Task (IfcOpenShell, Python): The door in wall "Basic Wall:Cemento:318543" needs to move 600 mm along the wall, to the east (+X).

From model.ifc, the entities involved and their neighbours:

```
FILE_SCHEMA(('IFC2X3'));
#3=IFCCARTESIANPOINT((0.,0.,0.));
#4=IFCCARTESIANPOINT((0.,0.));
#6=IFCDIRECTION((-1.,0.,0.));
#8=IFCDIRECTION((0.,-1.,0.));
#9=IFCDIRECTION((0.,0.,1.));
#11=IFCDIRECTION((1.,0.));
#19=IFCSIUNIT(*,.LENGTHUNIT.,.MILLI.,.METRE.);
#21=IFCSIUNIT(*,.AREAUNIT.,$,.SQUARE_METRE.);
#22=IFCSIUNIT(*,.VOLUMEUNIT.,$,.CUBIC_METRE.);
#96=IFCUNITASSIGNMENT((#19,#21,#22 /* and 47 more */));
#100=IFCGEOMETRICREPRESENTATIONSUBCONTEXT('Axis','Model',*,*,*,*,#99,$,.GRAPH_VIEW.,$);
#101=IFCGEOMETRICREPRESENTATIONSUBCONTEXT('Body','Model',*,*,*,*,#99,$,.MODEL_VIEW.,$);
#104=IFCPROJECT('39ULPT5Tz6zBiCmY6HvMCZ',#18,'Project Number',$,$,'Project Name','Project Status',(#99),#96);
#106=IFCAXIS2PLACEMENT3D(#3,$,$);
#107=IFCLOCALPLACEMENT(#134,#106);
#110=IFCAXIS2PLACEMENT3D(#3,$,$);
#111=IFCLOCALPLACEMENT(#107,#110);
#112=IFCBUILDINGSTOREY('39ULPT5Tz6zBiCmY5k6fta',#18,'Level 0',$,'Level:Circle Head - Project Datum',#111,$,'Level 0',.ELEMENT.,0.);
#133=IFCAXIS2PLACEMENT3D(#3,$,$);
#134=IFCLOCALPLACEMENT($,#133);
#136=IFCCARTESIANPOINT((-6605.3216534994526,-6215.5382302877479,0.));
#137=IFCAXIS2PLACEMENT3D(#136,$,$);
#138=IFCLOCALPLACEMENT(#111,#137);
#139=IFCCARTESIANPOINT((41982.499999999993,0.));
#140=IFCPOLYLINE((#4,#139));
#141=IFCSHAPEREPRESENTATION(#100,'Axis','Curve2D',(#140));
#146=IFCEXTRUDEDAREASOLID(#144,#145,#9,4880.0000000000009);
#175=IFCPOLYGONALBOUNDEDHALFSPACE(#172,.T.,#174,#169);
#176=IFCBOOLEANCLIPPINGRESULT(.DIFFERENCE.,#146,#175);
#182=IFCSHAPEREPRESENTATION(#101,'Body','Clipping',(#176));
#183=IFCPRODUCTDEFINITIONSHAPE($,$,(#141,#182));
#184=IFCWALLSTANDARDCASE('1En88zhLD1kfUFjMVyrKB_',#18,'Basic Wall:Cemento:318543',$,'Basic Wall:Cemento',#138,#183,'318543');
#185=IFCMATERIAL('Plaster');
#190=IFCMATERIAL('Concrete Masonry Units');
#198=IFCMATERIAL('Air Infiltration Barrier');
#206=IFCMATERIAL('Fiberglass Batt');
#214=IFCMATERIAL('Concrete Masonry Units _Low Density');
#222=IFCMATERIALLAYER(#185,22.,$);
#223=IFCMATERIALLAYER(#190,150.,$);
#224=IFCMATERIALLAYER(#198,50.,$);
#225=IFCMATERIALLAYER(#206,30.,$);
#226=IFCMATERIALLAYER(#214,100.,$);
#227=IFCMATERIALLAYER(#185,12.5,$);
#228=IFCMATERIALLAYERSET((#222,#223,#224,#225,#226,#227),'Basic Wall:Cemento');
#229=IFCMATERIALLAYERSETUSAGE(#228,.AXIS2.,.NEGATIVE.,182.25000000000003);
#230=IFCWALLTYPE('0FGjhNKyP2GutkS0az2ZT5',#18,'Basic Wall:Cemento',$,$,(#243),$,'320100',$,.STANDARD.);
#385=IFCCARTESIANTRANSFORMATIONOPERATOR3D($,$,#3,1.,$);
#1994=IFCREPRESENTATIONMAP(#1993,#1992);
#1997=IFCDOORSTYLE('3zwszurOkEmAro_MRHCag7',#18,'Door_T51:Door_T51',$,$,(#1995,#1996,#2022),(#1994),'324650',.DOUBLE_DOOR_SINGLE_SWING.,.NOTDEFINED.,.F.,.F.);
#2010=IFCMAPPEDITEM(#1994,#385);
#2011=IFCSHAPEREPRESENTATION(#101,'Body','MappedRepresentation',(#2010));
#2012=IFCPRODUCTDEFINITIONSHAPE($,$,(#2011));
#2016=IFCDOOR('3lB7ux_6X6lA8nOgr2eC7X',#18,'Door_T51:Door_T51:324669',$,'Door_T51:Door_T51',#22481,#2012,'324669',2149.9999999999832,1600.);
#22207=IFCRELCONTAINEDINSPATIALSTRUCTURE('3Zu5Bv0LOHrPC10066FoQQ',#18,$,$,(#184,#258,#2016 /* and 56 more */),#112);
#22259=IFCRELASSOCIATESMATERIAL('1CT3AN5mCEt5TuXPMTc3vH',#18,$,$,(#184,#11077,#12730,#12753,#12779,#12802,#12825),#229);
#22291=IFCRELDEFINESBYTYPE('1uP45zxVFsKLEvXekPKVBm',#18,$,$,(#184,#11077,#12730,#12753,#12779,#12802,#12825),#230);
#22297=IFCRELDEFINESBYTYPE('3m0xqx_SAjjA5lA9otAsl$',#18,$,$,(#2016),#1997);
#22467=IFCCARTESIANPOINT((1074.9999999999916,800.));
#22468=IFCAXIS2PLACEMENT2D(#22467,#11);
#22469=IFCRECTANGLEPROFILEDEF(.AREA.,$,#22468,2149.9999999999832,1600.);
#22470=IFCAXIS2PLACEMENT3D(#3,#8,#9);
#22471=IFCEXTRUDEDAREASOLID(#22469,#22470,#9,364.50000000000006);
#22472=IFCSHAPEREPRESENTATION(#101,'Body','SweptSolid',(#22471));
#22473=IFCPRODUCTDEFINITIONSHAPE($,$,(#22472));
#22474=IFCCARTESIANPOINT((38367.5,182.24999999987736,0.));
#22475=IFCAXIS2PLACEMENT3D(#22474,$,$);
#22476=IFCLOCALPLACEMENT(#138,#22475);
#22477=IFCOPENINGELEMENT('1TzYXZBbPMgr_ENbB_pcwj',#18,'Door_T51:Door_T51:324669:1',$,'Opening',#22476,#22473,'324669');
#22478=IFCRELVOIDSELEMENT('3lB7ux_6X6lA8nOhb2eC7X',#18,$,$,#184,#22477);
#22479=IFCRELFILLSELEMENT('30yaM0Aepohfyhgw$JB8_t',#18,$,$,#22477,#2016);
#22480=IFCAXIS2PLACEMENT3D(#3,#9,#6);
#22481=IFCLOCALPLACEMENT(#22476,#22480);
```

```python
import ifcopenshell
import ifcopenshell.api.geometry
import ifcopenshell.util.placement
import ifcopenshell.util.unit

model = ifcopenshell.open("model.ifc")
unit_scale = ifcopenshell.util.unit.calculate_unit_scale(model)

door = model.by_guid("3lB7ux_6X6lA8nOgr2eC7X")
opening = door.FillsVoids[0].RelatingOpeningElement
wall = opening.VoidsElements[0].RelatingBuildingElement

wall_matrix = ifcopenshell.util.placement.get_local_placement(wall.ObjectPlacement)
shift = wall_matrix[:3, 0] * 0.6 / unit_scale
before = ifcopenshell.util.placement.get_local_placement(door.ObjectPlacement)[:3, 3].copy()

# The door is placed relative to its opening, so it follows when the opening moves.
matrix = ifcopenshell.util.placement.get_local_placement(opening.ObjectPlacement)
matrix[:3, 3] += shift
ifcopenshell.api.geometry.edit_object_placement(
    model, product=opening, matrix=matrix, is_si=False, should_transform_children=True
)

after = ifcopenshell.util.placement.get_local_placement(door.ObjectPlacement)[:3, 3]
print("door moved by", (after - before).round(3) + 0.0)

model.write("model-out.ifc")
```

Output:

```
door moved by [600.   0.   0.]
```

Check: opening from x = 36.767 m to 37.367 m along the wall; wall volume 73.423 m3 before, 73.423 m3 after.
